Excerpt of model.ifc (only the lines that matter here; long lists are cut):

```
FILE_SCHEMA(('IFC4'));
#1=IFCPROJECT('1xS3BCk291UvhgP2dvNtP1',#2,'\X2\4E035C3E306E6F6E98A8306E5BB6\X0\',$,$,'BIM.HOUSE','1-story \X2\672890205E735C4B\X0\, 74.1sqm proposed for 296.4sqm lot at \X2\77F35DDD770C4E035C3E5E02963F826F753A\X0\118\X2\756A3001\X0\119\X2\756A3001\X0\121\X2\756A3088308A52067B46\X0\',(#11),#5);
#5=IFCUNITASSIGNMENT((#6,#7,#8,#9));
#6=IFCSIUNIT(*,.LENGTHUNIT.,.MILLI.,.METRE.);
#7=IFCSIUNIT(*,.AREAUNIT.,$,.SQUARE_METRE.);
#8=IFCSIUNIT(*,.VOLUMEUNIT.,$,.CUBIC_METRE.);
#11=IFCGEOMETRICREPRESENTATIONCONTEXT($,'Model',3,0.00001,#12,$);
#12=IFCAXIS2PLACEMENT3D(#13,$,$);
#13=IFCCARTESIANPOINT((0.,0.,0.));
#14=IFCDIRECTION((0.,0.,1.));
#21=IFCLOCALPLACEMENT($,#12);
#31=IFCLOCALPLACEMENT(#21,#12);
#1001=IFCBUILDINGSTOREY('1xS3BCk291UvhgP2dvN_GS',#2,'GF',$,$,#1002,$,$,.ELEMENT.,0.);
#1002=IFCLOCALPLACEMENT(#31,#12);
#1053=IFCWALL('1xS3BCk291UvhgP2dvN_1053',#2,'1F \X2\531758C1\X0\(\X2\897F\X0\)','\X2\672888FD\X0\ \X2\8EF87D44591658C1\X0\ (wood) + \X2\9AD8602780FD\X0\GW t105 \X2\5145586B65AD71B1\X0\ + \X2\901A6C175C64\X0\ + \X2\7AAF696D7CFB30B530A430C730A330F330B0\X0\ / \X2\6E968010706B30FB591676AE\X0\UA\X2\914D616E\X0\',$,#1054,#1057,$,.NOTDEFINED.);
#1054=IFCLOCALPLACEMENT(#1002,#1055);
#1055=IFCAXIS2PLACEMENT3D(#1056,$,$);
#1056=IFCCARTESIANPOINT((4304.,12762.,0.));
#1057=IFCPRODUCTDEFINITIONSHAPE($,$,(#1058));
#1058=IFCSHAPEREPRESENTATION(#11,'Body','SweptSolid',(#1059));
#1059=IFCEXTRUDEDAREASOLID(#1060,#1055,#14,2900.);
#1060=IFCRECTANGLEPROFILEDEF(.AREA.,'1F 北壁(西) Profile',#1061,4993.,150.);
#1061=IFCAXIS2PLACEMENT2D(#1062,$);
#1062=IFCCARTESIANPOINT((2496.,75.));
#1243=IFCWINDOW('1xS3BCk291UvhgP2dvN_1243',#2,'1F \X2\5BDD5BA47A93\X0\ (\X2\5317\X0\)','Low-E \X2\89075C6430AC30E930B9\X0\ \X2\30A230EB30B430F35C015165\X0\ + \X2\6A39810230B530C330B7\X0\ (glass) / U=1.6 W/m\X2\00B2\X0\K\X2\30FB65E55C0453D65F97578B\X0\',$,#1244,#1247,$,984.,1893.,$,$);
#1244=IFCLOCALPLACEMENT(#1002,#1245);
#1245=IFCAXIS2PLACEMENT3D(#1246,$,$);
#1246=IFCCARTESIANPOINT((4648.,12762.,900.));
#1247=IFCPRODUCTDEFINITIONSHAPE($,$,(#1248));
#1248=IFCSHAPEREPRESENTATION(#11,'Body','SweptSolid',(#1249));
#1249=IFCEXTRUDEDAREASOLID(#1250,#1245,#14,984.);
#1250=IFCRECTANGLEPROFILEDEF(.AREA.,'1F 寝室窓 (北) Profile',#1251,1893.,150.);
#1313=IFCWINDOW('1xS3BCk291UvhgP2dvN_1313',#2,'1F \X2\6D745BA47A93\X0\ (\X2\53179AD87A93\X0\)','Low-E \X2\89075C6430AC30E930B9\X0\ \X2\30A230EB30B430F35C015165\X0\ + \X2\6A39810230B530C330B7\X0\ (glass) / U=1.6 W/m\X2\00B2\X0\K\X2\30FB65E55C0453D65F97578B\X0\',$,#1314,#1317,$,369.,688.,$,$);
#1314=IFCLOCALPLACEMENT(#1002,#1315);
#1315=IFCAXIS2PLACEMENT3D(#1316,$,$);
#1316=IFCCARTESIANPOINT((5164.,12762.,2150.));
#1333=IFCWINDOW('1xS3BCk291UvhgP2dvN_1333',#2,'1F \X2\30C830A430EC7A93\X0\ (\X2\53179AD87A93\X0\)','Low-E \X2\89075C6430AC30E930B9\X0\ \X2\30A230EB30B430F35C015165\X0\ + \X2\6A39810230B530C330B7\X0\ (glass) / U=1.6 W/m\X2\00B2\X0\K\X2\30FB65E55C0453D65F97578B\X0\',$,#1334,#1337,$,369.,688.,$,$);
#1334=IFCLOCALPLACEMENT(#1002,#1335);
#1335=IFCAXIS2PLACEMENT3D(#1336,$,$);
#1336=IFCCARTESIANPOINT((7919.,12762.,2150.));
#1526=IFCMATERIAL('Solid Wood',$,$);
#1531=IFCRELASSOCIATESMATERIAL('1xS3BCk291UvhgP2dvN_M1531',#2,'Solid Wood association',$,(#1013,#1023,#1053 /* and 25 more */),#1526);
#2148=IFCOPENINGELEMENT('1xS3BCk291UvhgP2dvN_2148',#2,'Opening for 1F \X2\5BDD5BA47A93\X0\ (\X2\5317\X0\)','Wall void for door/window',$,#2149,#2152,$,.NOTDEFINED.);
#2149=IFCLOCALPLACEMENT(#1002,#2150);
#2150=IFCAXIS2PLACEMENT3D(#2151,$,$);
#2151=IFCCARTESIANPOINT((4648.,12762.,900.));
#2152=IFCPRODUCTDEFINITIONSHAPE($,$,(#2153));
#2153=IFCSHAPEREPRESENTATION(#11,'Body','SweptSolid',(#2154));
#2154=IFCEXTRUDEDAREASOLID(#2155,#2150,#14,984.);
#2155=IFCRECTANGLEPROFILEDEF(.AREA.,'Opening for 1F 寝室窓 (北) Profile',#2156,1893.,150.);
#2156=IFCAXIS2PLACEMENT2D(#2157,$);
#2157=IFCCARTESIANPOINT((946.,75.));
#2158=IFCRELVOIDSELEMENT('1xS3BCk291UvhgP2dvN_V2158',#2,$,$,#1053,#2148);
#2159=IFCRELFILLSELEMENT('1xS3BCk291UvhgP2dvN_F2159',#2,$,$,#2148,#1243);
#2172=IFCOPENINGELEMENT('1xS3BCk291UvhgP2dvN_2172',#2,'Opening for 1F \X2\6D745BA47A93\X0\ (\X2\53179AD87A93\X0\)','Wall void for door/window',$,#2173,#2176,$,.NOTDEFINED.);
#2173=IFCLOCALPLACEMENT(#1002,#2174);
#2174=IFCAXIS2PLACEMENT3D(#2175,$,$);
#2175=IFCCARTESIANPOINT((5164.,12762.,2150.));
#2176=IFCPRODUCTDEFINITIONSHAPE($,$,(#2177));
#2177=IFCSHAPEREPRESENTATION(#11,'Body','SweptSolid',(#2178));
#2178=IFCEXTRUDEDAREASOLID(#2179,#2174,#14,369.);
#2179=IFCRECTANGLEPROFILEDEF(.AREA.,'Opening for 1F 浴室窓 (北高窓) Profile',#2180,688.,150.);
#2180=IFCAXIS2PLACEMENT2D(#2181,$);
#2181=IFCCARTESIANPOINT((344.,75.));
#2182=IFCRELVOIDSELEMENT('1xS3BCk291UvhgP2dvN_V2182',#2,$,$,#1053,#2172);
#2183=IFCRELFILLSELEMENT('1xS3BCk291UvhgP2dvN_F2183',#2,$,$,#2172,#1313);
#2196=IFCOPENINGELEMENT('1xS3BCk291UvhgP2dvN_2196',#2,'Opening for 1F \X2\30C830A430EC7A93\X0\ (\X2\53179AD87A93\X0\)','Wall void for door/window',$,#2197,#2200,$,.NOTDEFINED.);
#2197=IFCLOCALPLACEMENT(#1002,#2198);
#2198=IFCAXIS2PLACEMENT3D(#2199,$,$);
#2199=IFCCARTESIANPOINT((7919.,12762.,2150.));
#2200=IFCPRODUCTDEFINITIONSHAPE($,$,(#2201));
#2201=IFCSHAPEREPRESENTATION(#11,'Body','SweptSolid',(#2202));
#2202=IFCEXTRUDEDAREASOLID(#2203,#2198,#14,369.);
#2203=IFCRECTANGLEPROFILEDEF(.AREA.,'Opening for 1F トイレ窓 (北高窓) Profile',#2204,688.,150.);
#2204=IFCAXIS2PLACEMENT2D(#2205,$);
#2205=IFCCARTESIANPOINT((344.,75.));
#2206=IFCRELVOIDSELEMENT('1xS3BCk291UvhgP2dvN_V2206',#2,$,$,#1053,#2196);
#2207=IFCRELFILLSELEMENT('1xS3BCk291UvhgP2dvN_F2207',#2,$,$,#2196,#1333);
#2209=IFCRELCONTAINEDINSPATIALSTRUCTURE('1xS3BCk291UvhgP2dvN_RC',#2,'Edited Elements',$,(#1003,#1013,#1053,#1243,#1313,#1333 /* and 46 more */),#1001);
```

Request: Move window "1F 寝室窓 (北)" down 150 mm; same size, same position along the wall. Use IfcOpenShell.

```python
import numpy as np
import ifcopenshell
import ifcopenshell.api.geometry
import ifcopenshell.util.placement
import ifcopenshell.util.unit

model = ifcopenshell.open("model.ifc")
unit_scale = ifcopenshell.util.unit.calculate_unit_scale(model)

window = model.by_guid("1xS3BCk291UvhgP2dvN_1243")
opening = window.FillsVoids[0].RelatingOpeningElement
dz = -0.15 / unit_scale

shift = np.array([0.0, 0.0, dz])
# The window is not placed relative to its opening, so move both.
for product in (opening, window):
    matrix = ifcopenshell.util.placement.get_local_placement(product.ObjectPlacement)
    matrix[:3, 3] += shift
    ifcopenshell.api.geometry.edit_object_placement(model, product=product, matrix=matrix, is_si=False)

print(f"moved by {dz * unit_scale:+.3f} m")

model.write("model_v2.ifc")
```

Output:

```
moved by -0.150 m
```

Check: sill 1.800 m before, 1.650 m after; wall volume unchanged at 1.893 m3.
